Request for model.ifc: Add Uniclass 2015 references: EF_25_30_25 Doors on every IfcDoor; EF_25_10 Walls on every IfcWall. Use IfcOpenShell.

First a look at what the model holds.

```python
import ifcopenshell

model = ifcopenshell.open("model.ifc")
print(model.schema)
print("classifications:", [c.Name for c in model.by_type("IfcClassification")])
for ifc_class in ("IfcDoor", "IfcRoof", "IfcStair", "IfcWall", "IfcWindow"):
    print(ifc_class, len(model.by_type(ifc_class)))
```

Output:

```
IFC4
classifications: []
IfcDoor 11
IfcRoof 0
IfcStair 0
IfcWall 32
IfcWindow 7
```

```python
import ifcopenshell
import ifcopenshell.api.classification

model = ifcopenshell.open("model.ifc")

system = ifcopenshell.api.classification.add_classification(model, classification="Uniclass 2015")

codes = {
    "IfcDoor": ("EF_25_30_25", "Doors"),
    "IfcWall": ("EF_25_10", "Walls"),
}
for ifc_class, (code, name) in codes.items():
    products = model.by_type(ifc_class)
    ifcopenshell.api.classification.add_reference(
        model, products=products, classification=system, identification=code, name=name
    )
    print(code, len(products))

model.write("model_rev.ifc")
```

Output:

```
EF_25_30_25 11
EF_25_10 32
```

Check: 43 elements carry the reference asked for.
